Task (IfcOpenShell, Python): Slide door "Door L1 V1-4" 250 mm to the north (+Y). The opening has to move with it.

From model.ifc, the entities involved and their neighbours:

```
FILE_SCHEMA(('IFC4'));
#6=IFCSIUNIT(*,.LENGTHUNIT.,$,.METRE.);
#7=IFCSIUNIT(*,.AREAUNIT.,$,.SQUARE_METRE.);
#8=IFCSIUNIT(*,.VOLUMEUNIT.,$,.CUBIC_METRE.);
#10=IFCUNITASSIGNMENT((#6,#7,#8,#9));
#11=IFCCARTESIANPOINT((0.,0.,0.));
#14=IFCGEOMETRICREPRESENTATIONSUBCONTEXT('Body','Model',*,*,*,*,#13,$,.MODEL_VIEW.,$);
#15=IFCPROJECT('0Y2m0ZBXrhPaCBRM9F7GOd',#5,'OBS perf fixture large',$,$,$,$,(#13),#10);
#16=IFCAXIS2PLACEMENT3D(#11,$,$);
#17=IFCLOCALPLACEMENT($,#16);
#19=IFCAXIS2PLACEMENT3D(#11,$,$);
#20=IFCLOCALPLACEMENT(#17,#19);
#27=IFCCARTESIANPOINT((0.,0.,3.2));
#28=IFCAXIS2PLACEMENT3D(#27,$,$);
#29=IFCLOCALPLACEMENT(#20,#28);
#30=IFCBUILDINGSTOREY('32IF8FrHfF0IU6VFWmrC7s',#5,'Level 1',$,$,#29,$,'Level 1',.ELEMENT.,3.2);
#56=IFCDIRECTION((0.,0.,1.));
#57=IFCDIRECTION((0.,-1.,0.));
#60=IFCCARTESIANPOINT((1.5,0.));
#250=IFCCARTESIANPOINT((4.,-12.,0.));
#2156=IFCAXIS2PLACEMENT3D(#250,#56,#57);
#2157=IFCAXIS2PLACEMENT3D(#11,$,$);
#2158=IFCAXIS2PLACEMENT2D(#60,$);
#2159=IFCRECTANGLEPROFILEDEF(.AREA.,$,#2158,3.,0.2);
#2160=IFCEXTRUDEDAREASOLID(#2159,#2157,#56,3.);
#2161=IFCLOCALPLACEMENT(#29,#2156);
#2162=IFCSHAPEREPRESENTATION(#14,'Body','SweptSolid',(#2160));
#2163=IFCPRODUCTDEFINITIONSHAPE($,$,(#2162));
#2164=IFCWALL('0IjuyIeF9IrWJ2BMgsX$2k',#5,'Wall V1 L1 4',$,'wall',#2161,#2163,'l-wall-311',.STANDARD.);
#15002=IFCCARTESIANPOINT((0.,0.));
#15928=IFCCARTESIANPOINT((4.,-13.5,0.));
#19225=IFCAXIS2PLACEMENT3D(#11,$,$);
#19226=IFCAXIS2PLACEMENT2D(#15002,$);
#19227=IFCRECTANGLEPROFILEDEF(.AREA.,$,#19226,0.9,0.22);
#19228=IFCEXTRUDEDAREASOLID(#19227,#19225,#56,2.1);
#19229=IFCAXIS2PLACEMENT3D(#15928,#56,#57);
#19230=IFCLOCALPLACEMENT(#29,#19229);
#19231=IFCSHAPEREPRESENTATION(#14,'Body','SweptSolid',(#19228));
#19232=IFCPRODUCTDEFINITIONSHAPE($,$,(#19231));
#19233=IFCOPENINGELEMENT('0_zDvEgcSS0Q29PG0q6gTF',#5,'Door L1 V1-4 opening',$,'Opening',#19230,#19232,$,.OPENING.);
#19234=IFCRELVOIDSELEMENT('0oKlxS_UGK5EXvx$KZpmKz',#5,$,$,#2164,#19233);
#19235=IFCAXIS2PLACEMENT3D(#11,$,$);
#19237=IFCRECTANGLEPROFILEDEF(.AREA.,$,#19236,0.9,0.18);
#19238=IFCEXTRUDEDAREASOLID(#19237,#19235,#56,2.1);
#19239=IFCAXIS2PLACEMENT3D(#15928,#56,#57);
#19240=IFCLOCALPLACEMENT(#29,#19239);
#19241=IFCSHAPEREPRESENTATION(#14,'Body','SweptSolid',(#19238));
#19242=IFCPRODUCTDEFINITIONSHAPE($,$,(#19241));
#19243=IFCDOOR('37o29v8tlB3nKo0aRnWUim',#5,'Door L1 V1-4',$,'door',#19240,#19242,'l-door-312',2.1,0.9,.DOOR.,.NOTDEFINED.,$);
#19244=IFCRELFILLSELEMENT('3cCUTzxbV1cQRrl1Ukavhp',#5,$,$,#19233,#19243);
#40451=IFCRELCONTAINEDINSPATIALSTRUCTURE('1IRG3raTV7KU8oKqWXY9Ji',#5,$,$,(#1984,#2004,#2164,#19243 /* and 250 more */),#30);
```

```python
import ifcopenshell
import ifcopenshell.api.geometry
import ifcopenshell.util.placement

model = ifcopenshell.open("model.ifc")

door = model.by_guid("37o29v8tlB3nKo0aRnWUim")
opening = door.FillsVoids[0].RelatingOpeningElement
wall = opening.VoidsElements[0].RelatingBuildingElement

wall_matrix = ifcopenshell.util.placement.get_local_placement(wall.ObjectPlacement)
shift = wall_matrix[:3, 0] * -0.25
before = ifcopenshell.util.placement.get_local_placement(door.ObjectPlacement)[:3, 3].copy()

# The door is not placed relative to its opening, so move both.
for product in (opening, door):
    matrix = ifcopenshell.util.placement.get_local_placement(product.ObjectPlacement)
    matrix[:3, 3] += shift
    ifcopenshell.api.geometry.edit_object_placement(model, product=product, matrix=matrix, is_si=False)

after = ifcopenshell.util.placement.get_local_placement(door.ObjectPlacement)[:3, 3]
print("door moved by", (after - before).round(3) + 0.0)

model.write("model_edited.ifc")
```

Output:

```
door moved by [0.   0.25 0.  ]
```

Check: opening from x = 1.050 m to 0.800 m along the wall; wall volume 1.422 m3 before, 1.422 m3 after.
